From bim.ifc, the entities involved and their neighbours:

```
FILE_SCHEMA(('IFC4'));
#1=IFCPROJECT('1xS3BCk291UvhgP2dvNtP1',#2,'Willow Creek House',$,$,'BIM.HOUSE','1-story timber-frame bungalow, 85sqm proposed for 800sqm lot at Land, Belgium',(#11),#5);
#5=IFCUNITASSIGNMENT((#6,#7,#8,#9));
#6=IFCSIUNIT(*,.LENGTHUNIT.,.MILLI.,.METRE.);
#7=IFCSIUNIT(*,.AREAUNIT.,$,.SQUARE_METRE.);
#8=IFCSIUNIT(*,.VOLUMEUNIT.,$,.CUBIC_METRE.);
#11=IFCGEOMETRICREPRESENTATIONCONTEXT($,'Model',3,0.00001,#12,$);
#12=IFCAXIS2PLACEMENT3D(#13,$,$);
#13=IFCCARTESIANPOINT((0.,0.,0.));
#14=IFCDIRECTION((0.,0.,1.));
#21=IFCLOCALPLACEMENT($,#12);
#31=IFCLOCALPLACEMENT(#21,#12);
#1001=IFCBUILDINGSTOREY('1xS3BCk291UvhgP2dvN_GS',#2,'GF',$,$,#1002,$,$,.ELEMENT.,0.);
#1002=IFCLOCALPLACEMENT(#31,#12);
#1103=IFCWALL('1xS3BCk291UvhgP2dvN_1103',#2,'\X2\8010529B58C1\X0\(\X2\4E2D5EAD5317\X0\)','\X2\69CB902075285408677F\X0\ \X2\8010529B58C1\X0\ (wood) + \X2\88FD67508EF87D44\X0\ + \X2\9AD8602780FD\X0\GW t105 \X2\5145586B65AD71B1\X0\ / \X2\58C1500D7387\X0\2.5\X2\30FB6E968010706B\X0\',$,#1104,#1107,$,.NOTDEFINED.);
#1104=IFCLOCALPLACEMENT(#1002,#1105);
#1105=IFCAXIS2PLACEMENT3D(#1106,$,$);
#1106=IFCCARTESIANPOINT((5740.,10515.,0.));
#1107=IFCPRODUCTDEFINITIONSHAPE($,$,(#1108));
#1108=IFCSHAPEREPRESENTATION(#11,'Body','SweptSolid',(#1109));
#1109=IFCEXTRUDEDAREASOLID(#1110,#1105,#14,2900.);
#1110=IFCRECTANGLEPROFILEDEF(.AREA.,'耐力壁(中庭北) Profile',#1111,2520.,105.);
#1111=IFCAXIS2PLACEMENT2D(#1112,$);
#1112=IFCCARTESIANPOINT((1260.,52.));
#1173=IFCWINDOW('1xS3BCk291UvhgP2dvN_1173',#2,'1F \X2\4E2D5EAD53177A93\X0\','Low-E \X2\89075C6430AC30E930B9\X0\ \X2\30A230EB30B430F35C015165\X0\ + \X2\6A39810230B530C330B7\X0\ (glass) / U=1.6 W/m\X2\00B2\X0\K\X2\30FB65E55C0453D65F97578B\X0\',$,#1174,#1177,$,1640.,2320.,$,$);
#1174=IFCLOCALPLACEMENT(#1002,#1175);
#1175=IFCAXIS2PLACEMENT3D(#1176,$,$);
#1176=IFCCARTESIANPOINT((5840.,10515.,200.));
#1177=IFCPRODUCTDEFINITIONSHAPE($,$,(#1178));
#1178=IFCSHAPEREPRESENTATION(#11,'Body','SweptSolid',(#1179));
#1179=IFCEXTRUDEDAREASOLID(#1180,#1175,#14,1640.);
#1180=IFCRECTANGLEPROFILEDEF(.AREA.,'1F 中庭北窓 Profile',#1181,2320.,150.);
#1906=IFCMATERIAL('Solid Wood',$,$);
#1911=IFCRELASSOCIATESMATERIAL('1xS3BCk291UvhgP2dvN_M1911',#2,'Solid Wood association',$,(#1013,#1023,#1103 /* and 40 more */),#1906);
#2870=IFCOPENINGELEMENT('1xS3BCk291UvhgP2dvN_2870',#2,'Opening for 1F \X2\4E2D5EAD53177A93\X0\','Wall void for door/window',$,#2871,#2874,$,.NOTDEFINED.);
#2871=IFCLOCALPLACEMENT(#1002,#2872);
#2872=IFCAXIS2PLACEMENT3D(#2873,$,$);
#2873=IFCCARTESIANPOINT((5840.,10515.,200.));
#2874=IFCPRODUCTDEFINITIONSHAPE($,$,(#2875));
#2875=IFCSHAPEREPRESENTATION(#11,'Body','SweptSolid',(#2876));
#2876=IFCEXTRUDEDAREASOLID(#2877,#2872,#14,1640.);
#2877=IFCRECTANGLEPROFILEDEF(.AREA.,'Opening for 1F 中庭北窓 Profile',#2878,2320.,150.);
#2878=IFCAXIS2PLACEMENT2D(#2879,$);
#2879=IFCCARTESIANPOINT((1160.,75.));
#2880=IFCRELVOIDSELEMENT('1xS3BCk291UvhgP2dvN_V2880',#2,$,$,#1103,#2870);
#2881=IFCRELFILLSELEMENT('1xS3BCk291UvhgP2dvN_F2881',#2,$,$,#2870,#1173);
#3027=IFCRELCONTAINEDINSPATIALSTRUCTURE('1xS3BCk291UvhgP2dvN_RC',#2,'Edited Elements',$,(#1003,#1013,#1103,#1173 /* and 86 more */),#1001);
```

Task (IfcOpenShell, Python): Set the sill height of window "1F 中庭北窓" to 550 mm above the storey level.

```python
import numpy as np
import ifcopenshell
import ifcopenshell.api.geometry
import ifcopenshell.geom
import ifcopenshell.util.element
import ifcopenshell.util.placement
import ifcopenshell.util.shape
import ifcopenshell.util.unit

model = ifcopenshell.open("bim.ifc")
unit_scale = ifcopenshell.util.unit.calculate_unit_scale(model)

window = model.by_id(1173)
opening = window.FillsVoids[0].RelatingOpeningElement
storey = ifcopenshell.util.element.get_container(window, ifc_class="IfcBuildingStorey")
level = ifcopenshell.util.placement.get_local_placement(storey.ObjectPlacement)[2, 3]

# The opening's origin need not be at the sill, so measure its lowest point.
shape = ifcopenshell.geom.create_shape(ifcopenshell.geom.settings(), opening)
bottom = ifcopenshell.util.shape.get_shape_bottom_elevation(shape, shape.geometry) / unit_scale
dz = level + 550.0 - bottom

shift = np.array([0.0, 0.0, dz])
# The window is not placed relative to its opening, so move both.
for product in (opening, window):
    matrix = ifcopenshell.util.placement.get_local_placement(product.ObjectPlacement)
    matrix[:3, 3] += shift
    ifcopenshell.api.geometry.edit_object_placement(model, product=product, matrix=matrix, is_si=False)

print(f"moved by {dz * unit_scale:+.3f} m")

model.write("bim_rev.ifc")
```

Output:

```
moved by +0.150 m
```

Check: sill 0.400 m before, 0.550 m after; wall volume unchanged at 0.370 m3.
